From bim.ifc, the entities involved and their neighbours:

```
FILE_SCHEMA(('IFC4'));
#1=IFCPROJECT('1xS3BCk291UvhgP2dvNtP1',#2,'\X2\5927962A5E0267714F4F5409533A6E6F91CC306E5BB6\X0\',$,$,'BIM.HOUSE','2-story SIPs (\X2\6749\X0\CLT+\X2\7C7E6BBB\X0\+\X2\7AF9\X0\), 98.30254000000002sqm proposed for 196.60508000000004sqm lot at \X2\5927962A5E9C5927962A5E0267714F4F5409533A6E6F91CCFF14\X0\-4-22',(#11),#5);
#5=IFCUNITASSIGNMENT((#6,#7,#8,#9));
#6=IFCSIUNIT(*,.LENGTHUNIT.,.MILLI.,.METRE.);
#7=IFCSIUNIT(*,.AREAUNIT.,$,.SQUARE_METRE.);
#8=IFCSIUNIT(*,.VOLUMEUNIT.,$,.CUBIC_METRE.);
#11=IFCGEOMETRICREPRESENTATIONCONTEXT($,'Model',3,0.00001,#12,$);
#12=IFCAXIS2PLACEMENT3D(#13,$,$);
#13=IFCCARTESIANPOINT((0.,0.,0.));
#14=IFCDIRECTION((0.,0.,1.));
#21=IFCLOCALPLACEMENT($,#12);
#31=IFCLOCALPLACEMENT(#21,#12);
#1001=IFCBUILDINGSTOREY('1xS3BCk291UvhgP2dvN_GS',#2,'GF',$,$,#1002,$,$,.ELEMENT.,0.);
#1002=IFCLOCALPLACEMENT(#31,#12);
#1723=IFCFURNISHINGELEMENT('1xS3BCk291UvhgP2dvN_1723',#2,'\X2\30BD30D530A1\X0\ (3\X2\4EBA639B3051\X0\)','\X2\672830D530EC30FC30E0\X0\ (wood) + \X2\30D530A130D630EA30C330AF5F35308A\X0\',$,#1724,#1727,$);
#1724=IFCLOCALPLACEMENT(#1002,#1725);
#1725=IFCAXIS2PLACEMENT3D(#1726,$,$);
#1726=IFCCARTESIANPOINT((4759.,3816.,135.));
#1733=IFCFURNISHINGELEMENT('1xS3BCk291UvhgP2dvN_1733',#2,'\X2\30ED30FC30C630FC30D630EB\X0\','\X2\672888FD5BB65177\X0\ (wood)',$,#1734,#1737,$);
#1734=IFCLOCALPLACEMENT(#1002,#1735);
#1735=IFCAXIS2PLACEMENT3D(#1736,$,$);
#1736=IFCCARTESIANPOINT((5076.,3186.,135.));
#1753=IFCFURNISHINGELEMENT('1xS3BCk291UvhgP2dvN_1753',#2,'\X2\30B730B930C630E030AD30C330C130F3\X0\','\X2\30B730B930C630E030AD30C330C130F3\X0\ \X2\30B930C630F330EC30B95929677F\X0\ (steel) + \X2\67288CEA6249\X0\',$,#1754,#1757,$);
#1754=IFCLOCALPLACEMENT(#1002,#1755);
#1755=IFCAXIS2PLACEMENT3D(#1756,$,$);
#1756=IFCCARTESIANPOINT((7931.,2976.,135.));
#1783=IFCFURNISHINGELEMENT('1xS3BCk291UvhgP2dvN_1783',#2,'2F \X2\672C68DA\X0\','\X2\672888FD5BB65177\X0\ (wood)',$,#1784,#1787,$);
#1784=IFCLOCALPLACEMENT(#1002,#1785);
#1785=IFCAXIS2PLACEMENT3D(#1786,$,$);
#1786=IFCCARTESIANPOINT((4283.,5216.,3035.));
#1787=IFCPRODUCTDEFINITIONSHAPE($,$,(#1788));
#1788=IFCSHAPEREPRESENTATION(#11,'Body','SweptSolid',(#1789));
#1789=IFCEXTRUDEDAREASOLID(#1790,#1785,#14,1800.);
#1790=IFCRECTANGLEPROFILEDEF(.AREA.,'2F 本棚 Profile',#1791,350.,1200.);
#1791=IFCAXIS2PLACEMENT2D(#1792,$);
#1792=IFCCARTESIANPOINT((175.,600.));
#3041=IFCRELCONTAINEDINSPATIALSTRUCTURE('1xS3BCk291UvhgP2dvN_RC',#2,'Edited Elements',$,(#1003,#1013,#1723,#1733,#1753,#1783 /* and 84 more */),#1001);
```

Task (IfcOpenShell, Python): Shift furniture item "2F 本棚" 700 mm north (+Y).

```python
import ifcopenshell
import ifcopenshell.api.geometry
import ifcopenshell.util.placement

model = ifcopenshell.open("bim.ifc")

item = model.by_id(1783)
matrix = ifcopenshell.util.placement.get_local_placement(item.ObjectPlacement)
matrix[1, 3] += 700.0
ifcopenshell.api.geometry.edit_object_placement(model, product=item, matrix=matrix, is_si=False)

print(ifcopenshell.util.placement.get_local_placement(item.ObjectPlacement).round(3) + 0.0)

model.write("bim_updated.ifc")
```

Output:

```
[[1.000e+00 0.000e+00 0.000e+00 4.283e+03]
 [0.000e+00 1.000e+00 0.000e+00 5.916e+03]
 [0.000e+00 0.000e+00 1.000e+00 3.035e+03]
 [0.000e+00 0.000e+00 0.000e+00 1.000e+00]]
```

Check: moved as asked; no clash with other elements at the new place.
